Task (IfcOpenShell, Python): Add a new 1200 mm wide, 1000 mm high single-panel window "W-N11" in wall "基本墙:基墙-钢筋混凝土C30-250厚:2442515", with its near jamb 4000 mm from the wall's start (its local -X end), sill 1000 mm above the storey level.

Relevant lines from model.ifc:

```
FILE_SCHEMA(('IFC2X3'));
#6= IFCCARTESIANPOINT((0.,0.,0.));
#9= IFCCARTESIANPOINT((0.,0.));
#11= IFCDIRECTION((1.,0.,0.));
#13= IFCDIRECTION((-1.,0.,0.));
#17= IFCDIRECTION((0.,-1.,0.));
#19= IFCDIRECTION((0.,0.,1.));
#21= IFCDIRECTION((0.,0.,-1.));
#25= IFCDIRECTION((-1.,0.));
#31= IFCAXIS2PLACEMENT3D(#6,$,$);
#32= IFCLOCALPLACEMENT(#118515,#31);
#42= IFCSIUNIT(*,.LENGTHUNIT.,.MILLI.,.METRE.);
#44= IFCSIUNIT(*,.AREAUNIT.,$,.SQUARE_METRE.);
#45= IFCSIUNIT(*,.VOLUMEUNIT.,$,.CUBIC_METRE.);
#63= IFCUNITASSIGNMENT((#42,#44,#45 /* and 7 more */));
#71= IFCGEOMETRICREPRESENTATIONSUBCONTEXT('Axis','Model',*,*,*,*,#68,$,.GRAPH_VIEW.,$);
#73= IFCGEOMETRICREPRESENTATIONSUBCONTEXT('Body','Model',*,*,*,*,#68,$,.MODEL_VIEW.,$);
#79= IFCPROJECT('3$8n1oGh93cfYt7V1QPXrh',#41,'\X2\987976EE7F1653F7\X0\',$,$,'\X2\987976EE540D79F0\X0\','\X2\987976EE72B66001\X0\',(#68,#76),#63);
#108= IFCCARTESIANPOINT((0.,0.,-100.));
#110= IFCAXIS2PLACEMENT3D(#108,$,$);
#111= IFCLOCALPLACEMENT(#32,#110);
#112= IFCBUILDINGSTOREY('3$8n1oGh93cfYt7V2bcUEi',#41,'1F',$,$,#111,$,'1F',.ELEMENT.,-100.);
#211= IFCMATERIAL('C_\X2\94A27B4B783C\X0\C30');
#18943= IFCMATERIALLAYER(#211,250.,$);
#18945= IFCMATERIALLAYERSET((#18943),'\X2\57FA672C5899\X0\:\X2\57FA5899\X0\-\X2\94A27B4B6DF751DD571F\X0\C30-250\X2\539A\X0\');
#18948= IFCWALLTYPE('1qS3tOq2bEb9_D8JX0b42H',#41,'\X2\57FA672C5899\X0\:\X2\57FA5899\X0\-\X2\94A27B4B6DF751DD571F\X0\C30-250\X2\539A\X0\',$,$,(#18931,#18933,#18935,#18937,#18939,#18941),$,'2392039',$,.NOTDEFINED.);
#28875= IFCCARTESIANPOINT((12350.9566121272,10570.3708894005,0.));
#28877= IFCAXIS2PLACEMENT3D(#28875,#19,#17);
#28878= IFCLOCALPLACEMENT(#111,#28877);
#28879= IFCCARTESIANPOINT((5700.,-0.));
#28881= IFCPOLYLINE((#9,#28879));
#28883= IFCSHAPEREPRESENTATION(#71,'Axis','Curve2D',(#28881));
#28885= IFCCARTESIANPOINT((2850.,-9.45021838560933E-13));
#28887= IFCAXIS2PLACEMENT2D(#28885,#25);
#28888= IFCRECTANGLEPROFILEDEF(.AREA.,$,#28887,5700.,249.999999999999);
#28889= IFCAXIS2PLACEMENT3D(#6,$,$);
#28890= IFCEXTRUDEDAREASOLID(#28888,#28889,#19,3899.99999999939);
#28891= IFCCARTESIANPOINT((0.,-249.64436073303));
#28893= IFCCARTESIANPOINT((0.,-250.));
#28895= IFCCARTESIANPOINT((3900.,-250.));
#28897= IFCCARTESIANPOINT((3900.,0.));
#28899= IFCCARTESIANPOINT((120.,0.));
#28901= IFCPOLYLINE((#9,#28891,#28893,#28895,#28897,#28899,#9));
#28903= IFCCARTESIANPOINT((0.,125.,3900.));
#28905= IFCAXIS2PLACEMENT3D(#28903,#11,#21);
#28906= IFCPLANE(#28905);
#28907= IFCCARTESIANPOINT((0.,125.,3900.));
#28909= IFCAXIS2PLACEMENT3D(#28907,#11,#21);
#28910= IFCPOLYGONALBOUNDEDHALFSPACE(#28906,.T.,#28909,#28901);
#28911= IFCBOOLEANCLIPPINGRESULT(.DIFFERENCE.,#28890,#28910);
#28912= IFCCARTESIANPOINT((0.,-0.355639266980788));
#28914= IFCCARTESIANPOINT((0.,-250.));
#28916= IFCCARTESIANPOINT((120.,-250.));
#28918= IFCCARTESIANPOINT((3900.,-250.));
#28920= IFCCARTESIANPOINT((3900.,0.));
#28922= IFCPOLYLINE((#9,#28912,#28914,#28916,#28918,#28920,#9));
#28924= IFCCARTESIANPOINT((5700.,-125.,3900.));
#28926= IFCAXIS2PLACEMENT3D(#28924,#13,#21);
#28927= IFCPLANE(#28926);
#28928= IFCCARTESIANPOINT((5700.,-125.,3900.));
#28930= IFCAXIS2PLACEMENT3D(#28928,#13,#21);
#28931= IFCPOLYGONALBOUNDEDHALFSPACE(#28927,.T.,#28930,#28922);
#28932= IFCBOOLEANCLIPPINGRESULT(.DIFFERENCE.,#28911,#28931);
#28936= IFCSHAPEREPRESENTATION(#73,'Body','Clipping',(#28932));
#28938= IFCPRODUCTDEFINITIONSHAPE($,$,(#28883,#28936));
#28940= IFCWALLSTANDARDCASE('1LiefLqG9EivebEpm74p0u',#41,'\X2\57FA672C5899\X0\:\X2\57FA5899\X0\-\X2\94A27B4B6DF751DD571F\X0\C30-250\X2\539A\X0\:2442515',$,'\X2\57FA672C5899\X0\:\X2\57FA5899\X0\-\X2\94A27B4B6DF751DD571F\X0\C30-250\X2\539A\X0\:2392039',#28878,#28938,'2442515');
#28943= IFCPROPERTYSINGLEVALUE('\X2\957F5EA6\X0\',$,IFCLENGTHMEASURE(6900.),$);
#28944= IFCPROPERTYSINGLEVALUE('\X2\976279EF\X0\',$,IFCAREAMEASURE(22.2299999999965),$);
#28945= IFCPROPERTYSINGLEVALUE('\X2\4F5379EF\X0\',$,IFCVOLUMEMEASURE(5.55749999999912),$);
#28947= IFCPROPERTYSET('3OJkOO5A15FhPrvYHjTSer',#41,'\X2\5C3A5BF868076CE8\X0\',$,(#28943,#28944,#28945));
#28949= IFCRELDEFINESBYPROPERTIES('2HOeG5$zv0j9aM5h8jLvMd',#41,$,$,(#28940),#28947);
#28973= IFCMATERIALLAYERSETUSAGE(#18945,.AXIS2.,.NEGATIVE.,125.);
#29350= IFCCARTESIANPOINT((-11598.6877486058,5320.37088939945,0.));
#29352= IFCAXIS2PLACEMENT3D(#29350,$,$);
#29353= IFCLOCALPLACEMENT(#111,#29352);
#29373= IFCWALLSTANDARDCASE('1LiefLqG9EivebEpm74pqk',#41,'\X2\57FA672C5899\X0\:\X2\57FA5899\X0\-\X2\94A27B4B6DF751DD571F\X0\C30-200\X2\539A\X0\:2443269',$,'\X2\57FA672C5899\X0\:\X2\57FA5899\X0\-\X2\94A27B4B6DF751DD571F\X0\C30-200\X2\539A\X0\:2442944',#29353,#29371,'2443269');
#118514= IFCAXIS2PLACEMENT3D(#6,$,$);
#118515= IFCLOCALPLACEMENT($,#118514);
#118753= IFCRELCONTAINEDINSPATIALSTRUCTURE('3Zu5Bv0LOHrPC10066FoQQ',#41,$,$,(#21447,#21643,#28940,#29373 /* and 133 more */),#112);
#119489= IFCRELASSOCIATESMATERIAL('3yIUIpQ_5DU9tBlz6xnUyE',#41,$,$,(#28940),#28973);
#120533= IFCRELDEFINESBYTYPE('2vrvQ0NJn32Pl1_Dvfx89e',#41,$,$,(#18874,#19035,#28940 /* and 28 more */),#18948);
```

```python
import numpy as np
import ifcopenshell
import ifcopenshell.api.feature
import ifcopenshell.api.geometry
import ifcopenshell.api.pset
import ifcopenshell.api.root
import ifcopenshell.api.spatial
import ifcopenshell.api.type
import ifcopenshell.geom
import ifcopenshell.util.element
import ifcopenshell.util.placement
import ifcopenshell.util.representation
import ifcopenshell.util.shape
import ifcopenshell.util.unit

model = ifcopenshell.open("model.ifc")
unit_scale = ifcopenshell.util.unit.calculate_unit_scale(model)
area_scale = ifcopenshell.util.unit.calculate_unit_scale(model, "AREAUNIT")
volume_scale = ifcopenshell.util.unit.calculate_unit_scale(model, "VOLUMEUNIT")
settings = ifcopenshell.geom.settings()


def volume(element):
    """Net volume in cubic metres, openings subtracted."""
    shape = ifcopenshell.geom.create_shape(settings, element)
    return ifcopenshell.util.shape.get_volume(shape.geometry)


wall = model.by_guid("1LiefLqG9EivebEpm74p0u")
storey = ifcopenshell.util.element.get_container(wall, ifc_class="IfcBuildingStorey")
context = ifcopenshell.util.representation.get_context(model, "Model", "Body", "MODEL_VIEW")
before = volume(wall)

width, height, from_end, sill = 1.2, 1, 4, 1  # metres

# The wall runs along its own X axis, and the end named is its -X end.
wall_shape = ifcopenshell.geom.create_shape(settings, wall)
x, y, z = ifcopenshell.util.shape.get_vertices(wall_shape.geometry).T
start = x.min() + from_end
face, thickness = float(y.min()), float(y.max() - y.min())
wall_matrix = ifcopenshell.util.placement.get_local_placement(wall.ObjectPlacement)
level = ifcopenshell.util.placement.get_local_placement(storey.ObjectPlacement)[2, 3]


def in_wall(x, y):
    """Placement at x, y metres in the wall's axes, at sill height."""
    matrix = wall_matrix.copy()
    matrix[:, 3] = wall_matrix @ np.array([x / unit_scale, y / unit_scale, 0.0, 1.0])
    matrix[2, 3] = level + sill / unit_scale
    return matrix


# Opening: a box that overshoots both wall faces by 50 mm.
opening = ifcopenshell.api.root.create_entity(model, ifc_class="IfcOpeningElement")
box = ifcopenshell.api.geometry.add_wall_representation(
    model, context=context, length=width, height=height, thickness=thickness + 0.1
)
ifcopenshell.api.geometry.assign_representation(model, product=opening, representation=box)
ifcopenshell.api.geometry.edit_object_placement(model, product=opening, matrix=in_wall(start, face - 0.05), is_si=False)
ifcopenshell.api.feature.add_feature(model, feature=opening, element=wall)

window = ifcopenshell.api.root.create_entity(model, ifc_class="IfcWindow", name="W-N11")
window.OverallWidth, window.OverallHeight = width / unit_scale, height / unit_scale
body = ifcopenshell.api.geometry.add_window_representation(
    model,
    context=context,
    overall_width=window.OverallWidth,
    overall_height=window.OverallHeight,
    partition_type="SINGLE_PANEL",
)
ifcopenshell.api.geometry.assign_representation(model, product=window, representation=body)
ifcopenshell.api.spatial.assign_container(model, products=[window], relating_structure=storey)
fills = ifcopenshell.api.feature.add_filling(model, opening=opening, element=window)
fills.OwnerHistory = window.OwnerHistory  # required in IFC2X3

# IFC2X3 keeps the operation on the window style.
style = ifcopenshell.api.root.create_entity(model, ifc_class="IfcWindowStyle", name="W-N11")
style.OperationType, style.ConstructionType = "SINGLE_PANEL", "NOTDEFINED"
style.ParameterTakesPrecedence = style.Sizeable = False
ifcopenshell.api.type.assign_type(model, related_objects=[window], relating_type=style)

# Centre the window in the wall's thickness.
ifcopenshell.api.geometry.edit_object_placement(model, product=window, matrix=in_wall(start, face), is_si=False)
window_shape = ifcopenshell.geom.create_shape(settings, window)
depth = ifcopenshell.util.shape.get_vertices(window_shape.geometry)[:, 1]
offset = face + thickness / 2 - (depth.min() + depth.max()) / 2
ifcopenshell.api.geometry.edit_object_placement(model, product=window, matrix=in_wall(start, offset), is_si=False)

after = volume(wall)

# Update the wall's stored quantities.
pset = model.by_id(ifcopenshell.util.element.get_pset(wall, "尺寸标注", should_inherit=False)["id"])
ifcopenshell.api.pset.edit_pset(model, pset=pset, properties={
    "面积": model.create_entity("IfcAreaMeasure", after / thickness / area_scale),
    "体积": model.create_entity("IfcVolumeMeasure", after / volume_scale),
})

print(f"wall volume {before:.3f} -> {after:.3f} m3")

model.write("model-out.ifc")
```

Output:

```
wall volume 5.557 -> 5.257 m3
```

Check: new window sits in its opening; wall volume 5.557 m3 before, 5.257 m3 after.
